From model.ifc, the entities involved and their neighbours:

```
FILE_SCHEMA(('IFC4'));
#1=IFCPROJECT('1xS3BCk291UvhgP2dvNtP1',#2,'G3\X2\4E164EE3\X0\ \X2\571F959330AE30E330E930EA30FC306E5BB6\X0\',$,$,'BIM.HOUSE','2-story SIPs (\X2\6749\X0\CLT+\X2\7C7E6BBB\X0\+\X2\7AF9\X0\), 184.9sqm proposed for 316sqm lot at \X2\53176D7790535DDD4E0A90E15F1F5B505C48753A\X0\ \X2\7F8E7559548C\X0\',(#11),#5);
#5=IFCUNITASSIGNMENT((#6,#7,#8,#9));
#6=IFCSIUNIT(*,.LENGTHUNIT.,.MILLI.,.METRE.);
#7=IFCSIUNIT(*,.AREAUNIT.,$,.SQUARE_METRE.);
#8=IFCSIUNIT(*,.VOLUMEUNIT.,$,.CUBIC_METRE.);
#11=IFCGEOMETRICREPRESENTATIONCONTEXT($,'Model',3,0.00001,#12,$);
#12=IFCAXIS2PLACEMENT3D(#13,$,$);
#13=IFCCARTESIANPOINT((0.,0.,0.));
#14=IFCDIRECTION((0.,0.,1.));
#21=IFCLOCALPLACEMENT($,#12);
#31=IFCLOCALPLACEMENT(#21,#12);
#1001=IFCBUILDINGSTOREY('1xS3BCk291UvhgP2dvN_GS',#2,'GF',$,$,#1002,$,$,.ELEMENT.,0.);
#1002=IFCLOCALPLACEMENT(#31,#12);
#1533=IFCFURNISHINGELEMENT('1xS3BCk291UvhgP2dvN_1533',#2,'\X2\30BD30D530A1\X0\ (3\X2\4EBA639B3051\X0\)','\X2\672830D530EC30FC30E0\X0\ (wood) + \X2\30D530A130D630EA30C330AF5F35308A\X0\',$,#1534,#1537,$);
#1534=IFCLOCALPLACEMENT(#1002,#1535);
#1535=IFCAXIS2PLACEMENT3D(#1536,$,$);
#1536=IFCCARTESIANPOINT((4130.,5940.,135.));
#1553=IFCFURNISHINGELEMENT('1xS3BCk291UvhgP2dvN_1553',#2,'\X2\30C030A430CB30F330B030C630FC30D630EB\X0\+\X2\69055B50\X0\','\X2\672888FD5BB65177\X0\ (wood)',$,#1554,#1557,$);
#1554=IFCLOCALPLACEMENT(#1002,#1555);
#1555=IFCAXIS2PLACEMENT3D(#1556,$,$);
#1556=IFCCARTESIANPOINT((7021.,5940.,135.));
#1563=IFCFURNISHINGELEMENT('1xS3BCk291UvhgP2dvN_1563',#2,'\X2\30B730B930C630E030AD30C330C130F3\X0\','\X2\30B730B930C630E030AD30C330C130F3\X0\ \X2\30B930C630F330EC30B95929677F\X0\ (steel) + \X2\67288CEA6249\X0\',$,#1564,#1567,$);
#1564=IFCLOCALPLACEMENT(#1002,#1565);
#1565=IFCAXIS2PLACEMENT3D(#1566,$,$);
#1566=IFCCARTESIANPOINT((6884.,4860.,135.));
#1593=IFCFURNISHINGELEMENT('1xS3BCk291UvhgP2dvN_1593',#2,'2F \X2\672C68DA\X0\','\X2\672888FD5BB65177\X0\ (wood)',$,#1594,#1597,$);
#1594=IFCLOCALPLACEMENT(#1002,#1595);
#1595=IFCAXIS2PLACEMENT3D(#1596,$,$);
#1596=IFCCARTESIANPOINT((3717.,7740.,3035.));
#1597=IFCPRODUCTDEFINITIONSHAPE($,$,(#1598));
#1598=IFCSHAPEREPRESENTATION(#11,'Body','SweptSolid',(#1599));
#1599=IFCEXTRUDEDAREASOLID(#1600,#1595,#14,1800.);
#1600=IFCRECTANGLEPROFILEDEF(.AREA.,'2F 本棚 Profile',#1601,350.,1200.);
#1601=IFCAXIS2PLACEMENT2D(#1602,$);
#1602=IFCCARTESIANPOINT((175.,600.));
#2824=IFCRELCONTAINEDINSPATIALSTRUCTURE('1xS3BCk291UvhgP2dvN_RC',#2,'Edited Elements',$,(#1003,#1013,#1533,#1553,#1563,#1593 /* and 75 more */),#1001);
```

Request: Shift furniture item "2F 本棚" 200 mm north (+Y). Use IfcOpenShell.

```python
import ifcopenshell
import ifcopenshell.api.geometry
import ifcopenshell.util.placement

model = ifcopenshell.open("model.ifc")

item = model.by_id(1593)
matrix = ifcopenshell.util.placement.get_local_placement(item.ObjectPlacement)
matrix[1, 3] += 200.0
ifcopenshell.api.geometry.edit_object_placement(model, product=item, matrix=matrix, is_si=False)

print(ifcopenshell.util.placement.get_local_placement(item.ObjectPlacement).round(3) + 0.0)

model.write("model_rev.ifc")
```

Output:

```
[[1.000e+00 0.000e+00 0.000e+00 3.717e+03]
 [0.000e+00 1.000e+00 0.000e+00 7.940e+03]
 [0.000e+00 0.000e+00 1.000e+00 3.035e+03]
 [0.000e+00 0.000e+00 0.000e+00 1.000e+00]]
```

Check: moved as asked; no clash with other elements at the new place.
